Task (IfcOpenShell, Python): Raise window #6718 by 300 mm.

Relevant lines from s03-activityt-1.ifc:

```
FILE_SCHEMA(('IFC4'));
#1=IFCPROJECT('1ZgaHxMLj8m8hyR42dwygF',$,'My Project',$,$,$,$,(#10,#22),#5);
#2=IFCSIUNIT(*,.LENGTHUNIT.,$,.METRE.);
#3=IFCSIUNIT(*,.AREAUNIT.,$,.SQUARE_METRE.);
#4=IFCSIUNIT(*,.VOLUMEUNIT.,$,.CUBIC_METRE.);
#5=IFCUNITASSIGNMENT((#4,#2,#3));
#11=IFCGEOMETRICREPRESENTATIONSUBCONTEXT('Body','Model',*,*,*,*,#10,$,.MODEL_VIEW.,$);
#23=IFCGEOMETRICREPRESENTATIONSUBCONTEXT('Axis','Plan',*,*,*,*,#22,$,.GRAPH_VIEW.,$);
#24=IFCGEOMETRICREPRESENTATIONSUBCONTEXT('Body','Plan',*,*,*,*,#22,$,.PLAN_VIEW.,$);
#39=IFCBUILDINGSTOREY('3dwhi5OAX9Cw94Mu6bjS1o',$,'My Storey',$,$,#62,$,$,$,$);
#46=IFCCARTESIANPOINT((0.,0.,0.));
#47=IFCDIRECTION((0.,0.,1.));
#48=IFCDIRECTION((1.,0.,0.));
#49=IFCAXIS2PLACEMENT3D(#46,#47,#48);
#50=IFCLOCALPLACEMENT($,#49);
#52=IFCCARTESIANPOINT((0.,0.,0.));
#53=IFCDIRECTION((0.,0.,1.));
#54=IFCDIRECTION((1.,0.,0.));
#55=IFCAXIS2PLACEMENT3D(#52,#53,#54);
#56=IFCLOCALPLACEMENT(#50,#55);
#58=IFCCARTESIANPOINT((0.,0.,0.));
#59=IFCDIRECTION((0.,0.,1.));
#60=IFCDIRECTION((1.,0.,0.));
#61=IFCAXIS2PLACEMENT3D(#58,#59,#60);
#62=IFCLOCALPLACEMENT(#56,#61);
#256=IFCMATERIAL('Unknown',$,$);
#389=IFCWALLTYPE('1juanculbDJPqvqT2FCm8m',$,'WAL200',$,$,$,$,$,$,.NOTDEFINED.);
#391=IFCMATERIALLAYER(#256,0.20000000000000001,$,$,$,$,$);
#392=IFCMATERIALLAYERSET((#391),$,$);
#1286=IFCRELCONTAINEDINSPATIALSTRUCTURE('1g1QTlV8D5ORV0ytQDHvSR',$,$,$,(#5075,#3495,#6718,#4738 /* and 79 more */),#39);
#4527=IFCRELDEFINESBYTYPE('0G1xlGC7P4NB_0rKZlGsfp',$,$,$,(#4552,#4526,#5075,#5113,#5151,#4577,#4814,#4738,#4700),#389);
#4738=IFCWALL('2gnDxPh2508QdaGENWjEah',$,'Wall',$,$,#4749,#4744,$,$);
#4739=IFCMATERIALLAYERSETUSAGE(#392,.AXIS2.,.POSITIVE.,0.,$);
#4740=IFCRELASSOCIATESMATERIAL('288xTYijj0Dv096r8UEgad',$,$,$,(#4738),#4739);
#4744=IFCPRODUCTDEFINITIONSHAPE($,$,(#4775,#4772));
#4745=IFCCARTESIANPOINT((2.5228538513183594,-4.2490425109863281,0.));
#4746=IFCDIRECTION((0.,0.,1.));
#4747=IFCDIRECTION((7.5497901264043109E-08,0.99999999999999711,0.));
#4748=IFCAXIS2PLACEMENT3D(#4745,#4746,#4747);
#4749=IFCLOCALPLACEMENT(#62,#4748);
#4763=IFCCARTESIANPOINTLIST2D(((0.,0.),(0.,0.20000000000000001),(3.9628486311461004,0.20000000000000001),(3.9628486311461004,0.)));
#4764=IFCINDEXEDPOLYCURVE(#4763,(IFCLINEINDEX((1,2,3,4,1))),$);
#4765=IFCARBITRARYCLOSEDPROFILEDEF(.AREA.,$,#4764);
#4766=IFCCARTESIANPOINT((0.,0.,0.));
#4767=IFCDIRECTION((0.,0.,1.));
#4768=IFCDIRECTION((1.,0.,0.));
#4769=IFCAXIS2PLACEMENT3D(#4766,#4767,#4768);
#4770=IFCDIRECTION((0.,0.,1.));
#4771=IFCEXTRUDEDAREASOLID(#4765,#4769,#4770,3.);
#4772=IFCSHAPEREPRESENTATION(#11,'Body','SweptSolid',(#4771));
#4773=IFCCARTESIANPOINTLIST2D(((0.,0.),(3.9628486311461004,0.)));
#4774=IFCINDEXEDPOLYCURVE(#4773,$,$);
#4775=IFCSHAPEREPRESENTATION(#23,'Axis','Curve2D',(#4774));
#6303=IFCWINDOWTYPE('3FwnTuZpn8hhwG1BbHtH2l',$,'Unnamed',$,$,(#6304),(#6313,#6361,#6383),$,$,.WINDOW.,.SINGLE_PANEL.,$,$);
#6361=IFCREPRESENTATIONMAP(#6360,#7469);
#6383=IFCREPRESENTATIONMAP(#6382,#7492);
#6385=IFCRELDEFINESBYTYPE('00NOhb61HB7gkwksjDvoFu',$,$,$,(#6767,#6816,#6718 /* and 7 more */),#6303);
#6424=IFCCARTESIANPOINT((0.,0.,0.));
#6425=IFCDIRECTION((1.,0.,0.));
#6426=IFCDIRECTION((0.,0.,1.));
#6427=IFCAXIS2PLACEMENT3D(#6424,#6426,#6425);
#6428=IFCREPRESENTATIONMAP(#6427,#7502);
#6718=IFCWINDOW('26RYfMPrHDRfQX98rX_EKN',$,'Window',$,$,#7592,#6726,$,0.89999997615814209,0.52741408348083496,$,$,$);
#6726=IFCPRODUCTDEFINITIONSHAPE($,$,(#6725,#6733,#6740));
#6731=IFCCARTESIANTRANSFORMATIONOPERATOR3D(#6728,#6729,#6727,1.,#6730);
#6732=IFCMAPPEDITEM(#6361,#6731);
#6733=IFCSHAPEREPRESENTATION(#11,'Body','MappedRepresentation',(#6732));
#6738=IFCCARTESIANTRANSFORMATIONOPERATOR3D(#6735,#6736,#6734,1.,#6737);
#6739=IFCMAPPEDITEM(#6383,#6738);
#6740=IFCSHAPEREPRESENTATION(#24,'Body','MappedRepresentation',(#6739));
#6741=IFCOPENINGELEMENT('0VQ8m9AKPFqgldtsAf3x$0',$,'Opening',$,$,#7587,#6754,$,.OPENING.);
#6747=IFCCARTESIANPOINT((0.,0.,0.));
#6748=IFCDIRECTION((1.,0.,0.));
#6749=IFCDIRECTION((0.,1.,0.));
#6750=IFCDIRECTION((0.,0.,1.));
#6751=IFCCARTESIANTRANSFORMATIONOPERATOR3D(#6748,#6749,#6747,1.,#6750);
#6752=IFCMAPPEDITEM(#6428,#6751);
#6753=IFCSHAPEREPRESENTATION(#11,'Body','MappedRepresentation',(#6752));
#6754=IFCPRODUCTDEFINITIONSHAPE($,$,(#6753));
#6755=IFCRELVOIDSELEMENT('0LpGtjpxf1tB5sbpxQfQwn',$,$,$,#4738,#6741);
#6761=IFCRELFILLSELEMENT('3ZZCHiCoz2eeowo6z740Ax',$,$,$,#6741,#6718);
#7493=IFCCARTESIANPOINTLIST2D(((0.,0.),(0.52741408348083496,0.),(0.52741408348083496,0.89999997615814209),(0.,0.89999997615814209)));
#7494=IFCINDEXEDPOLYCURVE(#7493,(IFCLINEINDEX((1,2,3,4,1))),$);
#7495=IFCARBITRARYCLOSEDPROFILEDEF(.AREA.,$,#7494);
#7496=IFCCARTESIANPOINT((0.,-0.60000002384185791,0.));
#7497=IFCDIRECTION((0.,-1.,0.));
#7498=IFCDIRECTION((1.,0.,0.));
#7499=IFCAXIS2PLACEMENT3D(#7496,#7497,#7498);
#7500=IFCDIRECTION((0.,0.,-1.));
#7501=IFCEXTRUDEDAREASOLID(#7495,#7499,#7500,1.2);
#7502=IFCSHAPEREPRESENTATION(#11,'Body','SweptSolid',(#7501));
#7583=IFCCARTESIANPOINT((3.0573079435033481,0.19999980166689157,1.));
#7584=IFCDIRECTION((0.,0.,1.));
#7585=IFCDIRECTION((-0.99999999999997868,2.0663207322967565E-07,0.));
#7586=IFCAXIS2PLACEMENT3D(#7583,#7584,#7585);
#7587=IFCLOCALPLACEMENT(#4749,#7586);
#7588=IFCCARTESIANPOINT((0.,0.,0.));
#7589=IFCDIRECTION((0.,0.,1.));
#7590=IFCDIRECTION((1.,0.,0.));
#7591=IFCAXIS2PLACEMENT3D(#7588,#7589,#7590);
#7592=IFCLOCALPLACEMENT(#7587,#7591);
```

```python
import numpy as np
import ifcopenshell
import ifcopenshell.api.geometry
import ifcopenshell.util.placement
import ifcopenshell.util.unit

model = ifcopenshell.open("s03-activityt-1.ifc")
unit_scale = ifcopenshell.util.unit.calculate_unit_scale(model)

window = model.by_id(6718)
opening = window.FillsVoids[0].RelatingOpeningElement
dz = 0.3 / unit_scale

shift = np.array([0.0, 0.0, dz])
# The window is placed relative to its opening, so it follows when the opening moves.
matrix = ifcopenshell.util.placement.get_local_placement(opening.ObjectPlacement)
matrix[:3, 3] += shift
ifcopenshell.api.geometry.edit_object_placement(
    model, product=opening, matrix=matrix, is_si=False, should_transform_children=True
)

print(f"moved by {dz * unit_scale:+.3f} m")

model.write("s03-activityt-1_updated.ifc")
```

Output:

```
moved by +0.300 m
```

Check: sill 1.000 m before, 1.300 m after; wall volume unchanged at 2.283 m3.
